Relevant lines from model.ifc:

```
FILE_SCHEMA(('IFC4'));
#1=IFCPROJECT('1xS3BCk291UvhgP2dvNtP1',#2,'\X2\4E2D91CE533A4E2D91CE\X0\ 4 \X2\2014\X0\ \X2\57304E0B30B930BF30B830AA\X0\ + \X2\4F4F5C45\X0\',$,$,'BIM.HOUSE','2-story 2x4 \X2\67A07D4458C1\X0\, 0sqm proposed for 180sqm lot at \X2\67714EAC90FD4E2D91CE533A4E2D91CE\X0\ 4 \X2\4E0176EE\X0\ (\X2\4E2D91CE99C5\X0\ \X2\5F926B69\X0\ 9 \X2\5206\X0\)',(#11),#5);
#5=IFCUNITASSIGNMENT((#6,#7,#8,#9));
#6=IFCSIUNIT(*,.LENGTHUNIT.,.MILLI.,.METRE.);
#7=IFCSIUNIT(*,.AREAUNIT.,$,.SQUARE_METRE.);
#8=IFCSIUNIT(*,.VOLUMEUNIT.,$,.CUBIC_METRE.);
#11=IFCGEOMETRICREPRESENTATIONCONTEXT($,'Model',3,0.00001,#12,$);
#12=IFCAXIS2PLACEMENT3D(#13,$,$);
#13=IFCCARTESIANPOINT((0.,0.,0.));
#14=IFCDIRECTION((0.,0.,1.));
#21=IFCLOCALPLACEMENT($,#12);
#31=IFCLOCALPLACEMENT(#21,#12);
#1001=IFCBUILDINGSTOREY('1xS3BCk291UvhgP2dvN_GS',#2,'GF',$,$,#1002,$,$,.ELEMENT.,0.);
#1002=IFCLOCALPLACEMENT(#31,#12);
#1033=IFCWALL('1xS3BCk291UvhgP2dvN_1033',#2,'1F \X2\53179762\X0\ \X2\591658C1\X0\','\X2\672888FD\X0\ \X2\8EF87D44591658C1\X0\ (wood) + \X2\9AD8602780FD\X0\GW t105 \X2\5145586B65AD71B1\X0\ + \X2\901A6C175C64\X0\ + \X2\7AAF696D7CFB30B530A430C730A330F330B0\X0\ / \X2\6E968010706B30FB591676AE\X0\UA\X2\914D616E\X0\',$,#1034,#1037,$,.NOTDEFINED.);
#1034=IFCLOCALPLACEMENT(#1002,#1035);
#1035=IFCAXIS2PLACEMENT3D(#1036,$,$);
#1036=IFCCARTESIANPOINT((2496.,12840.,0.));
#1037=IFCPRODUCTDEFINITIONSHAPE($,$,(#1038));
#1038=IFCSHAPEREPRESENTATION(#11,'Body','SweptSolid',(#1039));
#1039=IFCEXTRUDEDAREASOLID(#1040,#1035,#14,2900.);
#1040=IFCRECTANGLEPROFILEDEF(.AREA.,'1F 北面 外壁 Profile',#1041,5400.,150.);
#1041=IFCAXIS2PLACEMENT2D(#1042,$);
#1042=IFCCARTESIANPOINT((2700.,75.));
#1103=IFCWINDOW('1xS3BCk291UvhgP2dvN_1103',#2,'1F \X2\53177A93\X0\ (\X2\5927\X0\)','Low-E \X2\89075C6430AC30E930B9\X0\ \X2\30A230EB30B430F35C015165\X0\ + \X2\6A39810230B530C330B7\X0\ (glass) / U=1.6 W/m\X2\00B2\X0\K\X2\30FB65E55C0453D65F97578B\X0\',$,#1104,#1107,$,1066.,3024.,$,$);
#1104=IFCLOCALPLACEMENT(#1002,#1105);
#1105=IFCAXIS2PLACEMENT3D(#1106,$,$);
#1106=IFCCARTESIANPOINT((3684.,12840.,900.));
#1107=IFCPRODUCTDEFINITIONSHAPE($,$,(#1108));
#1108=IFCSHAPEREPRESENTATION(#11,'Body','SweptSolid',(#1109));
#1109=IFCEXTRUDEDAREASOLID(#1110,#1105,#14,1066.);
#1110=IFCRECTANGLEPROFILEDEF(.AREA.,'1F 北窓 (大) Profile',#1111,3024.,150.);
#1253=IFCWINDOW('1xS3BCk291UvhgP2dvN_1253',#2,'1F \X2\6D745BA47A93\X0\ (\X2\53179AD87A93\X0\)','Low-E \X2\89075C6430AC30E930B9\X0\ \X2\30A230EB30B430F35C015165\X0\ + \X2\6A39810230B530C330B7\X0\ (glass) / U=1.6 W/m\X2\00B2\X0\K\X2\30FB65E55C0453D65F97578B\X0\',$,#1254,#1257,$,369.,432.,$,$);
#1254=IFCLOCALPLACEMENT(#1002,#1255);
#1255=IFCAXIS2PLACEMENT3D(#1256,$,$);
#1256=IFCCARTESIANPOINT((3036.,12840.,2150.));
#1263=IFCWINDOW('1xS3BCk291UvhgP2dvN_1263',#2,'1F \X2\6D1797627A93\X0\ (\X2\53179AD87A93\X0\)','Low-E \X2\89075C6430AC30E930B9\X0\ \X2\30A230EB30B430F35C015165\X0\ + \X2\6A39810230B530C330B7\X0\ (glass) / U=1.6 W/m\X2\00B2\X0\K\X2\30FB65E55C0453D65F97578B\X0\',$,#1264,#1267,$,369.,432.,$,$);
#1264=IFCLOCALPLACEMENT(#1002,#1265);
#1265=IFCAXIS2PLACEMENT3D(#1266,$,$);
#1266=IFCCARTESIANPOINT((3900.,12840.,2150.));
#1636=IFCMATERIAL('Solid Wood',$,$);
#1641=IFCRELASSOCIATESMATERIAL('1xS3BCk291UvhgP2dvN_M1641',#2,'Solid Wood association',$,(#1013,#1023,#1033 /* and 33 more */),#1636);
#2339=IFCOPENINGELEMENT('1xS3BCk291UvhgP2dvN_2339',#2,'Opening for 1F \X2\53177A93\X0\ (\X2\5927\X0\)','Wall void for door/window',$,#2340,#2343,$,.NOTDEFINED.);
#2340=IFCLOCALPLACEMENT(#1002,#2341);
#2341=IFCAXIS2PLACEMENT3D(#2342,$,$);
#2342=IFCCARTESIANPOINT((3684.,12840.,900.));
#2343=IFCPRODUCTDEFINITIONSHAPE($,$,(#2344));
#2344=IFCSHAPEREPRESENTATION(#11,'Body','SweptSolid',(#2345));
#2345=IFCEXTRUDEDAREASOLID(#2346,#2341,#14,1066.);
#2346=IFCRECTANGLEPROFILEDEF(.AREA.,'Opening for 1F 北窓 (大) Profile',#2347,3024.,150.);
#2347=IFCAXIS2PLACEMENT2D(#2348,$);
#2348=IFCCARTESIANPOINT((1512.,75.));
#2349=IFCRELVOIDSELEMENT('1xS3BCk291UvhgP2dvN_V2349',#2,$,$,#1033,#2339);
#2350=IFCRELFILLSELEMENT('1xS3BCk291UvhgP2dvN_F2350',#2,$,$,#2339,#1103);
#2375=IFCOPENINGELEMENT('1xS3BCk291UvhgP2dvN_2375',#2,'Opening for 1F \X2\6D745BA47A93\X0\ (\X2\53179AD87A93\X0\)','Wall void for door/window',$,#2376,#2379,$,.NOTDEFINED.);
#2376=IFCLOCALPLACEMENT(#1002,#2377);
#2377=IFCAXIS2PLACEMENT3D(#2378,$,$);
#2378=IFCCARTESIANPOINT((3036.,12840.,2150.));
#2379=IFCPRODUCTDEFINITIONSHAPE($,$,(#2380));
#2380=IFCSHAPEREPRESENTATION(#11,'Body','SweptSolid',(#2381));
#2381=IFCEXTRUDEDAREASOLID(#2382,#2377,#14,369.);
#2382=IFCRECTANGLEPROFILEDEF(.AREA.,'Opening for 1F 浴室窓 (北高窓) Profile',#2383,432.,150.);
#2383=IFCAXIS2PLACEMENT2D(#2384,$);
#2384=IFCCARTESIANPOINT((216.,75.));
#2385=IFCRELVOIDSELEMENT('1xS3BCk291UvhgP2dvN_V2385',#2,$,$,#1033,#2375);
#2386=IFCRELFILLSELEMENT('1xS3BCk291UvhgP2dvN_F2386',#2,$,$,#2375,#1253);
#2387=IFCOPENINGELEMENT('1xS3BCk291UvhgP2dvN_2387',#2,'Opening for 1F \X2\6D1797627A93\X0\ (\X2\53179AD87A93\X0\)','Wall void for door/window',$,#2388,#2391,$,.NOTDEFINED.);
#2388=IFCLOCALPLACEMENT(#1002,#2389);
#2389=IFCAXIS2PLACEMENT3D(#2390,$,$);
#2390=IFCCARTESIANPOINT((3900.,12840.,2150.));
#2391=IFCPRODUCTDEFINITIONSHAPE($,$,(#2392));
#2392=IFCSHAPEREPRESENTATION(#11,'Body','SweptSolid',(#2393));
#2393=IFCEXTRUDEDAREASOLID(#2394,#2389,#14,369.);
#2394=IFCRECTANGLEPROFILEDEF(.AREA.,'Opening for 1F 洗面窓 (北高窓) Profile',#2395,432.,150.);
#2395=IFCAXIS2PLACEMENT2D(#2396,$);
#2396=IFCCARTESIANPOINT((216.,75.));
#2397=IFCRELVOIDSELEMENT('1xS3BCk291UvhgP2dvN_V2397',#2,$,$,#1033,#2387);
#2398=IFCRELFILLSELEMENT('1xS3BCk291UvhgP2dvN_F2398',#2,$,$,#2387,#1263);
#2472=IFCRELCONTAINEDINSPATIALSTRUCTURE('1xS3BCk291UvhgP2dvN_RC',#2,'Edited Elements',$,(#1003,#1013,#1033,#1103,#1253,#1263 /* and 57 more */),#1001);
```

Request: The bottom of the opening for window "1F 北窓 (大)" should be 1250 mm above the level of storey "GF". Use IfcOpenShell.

```python
import numpy as np
import ifcopenshell
import ifcopenshell.api.geometry
import ifcopenshell.geom
import ifcopenshell.util.element
import ifcopenshell.util.placement
import ifcopenshell.util.shape
import ifcopenshell.util.unit

model = ifcopenshell.open("model.ifc")
unit_scale = ifcopenshell.util.unit.calculate_unit_scale(model)

window = model.by_id(1103)
opening = window.FillsVoids[0].RelatingOpeningElement
storey = ifcopenshell.util.element.get_container(window, ifc_class="IfcBuildingStorey")
level = ifcopenshell.util.placement.get_local_placement(storey.ObjectPlacement)[2, 3]

# The opening's origin need not be at the sill, so measure its lowest point.
shape = ifcopenshell.geom.create_shape(ifcopenshell.geom.settings(), opening)
bottom = ifcopenshell.util.shape.get_shape_bottom_elevation(shape, shape.geometry) / unit_scale
dz = level + 1.25 / unit_scale - bottom

shift = np.array([0.0, 0.0, dz])
# The window is not placed relative to its opening, so move both.
for product in (opening, window):
    matrix = ifcopenshell.util.placement.get_local_placement(product.ObjectPlacement)
    matrix[:3, 3] += shift
    ifcopenshell.api.geometry.edit_object_placement(model, product=product, matrix=matrix, is_si=False)

print(f"moved by {dz * unit_scale:+.3f} m")

model.write("model_edited.ifc")
```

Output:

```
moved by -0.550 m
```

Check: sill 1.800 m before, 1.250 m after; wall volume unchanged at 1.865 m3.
